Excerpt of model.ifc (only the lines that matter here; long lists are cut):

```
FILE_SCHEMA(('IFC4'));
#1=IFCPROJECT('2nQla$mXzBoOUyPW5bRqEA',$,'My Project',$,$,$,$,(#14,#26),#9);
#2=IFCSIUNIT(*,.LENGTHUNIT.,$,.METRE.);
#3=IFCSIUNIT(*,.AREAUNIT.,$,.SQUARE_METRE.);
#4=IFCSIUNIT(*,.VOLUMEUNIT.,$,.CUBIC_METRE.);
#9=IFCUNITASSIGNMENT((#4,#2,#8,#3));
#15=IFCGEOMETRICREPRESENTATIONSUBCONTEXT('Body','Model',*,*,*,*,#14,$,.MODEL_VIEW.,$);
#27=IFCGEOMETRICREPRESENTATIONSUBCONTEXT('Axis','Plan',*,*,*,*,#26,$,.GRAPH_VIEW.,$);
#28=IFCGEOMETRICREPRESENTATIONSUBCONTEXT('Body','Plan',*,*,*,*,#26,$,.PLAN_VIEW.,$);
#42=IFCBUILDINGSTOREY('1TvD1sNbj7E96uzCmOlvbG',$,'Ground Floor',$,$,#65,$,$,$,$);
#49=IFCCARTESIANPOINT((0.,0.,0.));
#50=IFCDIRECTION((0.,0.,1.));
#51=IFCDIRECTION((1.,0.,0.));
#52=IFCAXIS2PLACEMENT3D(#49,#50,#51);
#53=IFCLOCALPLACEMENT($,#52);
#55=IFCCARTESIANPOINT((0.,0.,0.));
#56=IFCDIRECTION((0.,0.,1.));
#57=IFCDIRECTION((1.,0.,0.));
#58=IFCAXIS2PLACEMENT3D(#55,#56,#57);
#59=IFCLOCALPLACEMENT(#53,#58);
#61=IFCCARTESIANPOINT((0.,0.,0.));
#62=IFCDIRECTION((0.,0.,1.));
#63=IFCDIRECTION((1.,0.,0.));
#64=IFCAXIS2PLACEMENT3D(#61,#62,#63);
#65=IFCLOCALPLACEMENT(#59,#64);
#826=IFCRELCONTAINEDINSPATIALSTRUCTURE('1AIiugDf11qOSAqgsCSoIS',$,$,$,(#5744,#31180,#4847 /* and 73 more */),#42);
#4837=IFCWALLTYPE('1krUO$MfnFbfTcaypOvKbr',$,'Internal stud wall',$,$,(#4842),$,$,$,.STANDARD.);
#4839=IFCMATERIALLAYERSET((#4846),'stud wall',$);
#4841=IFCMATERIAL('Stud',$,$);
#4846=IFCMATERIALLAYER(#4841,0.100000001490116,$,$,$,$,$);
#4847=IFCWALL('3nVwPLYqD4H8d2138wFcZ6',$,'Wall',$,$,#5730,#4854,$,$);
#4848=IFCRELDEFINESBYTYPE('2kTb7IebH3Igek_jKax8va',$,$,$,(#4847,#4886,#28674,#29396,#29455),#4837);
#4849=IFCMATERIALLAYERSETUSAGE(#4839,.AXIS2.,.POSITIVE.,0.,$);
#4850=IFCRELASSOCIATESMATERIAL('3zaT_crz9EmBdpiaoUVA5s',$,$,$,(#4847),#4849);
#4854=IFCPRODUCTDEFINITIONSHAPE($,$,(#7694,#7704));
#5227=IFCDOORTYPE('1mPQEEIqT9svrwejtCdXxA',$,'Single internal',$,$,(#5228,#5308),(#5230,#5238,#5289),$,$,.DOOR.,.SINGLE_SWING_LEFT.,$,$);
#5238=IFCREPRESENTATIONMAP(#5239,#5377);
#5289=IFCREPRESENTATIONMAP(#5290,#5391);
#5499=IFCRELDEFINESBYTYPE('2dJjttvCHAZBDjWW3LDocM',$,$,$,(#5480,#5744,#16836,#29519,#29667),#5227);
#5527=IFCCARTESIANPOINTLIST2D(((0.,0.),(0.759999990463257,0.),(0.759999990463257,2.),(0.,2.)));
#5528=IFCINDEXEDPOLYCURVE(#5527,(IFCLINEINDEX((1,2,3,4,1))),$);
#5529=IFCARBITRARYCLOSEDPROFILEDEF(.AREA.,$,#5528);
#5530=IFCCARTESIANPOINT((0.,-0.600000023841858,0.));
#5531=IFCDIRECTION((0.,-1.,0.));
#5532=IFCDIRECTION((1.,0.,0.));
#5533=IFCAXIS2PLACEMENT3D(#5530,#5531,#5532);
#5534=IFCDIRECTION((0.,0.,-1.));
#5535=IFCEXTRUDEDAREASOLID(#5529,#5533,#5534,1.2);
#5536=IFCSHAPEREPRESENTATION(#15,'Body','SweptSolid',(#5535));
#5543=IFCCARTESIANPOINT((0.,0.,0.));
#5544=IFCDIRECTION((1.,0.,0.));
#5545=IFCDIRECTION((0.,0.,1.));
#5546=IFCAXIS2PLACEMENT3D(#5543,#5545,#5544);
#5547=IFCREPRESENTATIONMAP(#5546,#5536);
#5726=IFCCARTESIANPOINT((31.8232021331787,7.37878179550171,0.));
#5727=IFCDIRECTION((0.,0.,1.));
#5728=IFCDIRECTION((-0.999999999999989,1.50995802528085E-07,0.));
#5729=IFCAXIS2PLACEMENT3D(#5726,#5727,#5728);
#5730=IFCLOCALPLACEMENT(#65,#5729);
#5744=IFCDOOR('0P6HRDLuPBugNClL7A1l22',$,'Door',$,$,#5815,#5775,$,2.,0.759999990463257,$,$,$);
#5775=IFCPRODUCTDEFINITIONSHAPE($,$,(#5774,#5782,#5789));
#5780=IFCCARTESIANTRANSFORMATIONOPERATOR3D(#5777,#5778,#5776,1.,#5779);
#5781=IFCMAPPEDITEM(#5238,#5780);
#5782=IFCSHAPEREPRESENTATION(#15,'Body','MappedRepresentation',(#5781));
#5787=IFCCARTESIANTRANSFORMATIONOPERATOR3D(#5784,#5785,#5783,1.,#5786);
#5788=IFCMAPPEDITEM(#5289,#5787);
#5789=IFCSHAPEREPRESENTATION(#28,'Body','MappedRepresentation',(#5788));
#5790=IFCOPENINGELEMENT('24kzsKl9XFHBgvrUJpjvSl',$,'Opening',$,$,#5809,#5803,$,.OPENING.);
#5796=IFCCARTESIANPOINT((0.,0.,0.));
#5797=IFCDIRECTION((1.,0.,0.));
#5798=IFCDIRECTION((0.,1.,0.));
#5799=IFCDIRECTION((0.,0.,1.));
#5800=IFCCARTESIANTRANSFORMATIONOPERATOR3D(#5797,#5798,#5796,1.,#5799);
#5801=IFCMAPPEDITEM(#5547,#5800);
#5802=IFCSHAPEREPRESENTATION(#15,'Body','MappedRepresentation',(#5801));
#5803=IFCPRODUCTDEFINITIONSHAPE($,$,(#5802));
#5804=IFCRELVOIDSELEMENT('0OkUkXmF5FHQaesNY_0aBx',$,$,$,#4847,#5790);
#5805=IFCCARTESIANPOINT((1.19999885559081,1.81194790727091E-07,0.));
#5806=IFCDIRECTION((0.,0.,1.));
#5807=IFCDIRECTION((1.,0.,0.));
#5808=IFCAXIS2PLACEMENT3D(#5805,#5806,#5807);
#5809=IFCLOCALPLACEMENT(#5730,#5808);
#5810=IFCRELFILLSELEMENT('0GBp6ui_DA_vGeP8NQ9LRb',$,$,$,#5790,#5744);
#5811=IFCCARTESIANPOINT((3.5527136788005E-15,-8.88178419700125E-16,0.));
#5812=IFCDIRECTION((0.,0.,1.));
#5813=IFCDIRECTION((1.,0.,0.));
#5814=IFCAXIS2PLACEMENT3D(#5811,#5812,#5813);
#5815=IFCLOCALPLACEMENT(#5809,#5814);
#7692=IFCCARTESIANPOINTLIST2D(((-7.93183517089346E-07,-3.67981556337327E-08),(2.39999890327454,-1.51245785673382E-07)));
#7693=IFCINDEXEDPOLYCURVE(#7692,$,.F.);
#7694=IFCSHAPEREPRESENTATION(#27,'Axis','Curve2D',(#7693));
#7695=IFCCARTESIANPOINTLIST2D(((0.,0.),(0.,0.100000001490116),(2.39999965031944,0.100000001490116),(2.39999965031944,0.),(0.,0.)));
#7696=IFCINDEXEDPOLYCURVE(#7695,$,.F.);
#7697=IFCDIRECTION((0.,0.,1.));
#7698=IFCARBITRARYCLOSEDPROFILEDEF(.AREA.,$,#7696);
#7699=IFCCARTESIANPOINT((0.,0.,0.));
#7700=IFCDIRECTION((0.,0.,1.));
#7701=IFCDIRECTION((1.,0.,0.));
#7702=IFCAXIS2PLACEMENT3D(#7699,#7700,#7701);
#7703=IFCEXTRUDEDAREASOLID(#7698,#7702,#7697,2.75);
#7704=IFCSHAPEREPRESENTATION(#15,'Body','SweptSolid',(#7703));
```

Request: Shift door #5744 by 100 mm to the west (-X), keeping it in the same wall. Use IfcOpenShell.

```python
import ifcopenshell
import ifcopenshell.api.geometry
import ifcopenshell.util.placement
import ifcopenshell.util.unit

model = ifcopenshell.open("model.ifc")
unit_scale = ifcopenshell.util.unit.calculate_unit_scale(model)

door = model.by_id(5744)
opening = door.FillsVoids[0].RelatingOpeningElement
wall = opening.VoidsElements[0].RelatingBuildingElement

wall_matrix = ifcopenshell.util.placement.get_local_placement(wall.ObjectPlacement)
shift = wall_matrix[:3, 0] * 0.1 / unit_scale
before = ifcopenshell.util.placement.get_local_placement(door.ObjectPlacement)[:3, 3].copy()

# The door is placed relative to its opening, so it follows when the opening moves.
matrix = ifcopenshell.util.placement.get_local_placement(opening.ObjectPlacement)
matrix[:3, 3] += shift
ifcopenshell.api.geometry.edit_object_placement(
    model, product=opening, matrix=matrix, is_si=False, should_transform_children=True
)

after = ifcopenshell.util.placement.get_local_placement(door.ObjectPlacement)[:3, 3]
print("door moved by", (after - before).round(3) + 0.0)

model.write("model_edited.ifc")
```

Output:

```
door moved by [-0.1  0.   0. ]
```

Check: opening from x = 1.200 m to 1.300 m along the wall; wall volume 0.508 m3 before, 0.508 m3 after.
